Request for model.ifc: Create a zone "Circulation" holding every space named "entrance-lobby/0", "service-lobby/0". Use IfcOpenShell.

First a look at what the model holds.

```python
import ifcopenshell

model = ifcopenshell.open("model.ifc")
print(model.schema)
seen = {}
for space in model.by_type("IfcSpace"):
    seen[space.Name] = seen.get(space.Name, 0) + 1
for name, count in sorted(seen.items(), key=str):
    print(count, "x", name)
print("zones:", [z.Name for z in model.by_type("IfcZone")][:20])
```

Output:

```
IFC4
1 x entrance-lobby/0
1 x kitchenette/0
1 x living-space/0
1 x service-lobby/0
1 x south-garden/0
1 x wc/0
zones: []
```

```python
import ifcopenshell
import ifcopenshell.api.group
import ifcopenshell.api.root

model = ifcopenshell.open("model.ifc")

names = {"entrance-lobby/0", "service-lobby/0"}
spaces = [s for s in model.by_type("IfcSpace") if s.Name in names]

zone = ifcopenshell.api.root.create_entity(model, ifc_class="IfcZone", name="Circulation")
ifcopenshell.api.group.assign_group(model, products=spaces, group=zone)
print(len(spaces), "spaces in", zone.Name)

model.write("model_rev.ifc")
```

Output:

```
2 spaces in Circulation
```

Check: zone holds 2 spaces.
